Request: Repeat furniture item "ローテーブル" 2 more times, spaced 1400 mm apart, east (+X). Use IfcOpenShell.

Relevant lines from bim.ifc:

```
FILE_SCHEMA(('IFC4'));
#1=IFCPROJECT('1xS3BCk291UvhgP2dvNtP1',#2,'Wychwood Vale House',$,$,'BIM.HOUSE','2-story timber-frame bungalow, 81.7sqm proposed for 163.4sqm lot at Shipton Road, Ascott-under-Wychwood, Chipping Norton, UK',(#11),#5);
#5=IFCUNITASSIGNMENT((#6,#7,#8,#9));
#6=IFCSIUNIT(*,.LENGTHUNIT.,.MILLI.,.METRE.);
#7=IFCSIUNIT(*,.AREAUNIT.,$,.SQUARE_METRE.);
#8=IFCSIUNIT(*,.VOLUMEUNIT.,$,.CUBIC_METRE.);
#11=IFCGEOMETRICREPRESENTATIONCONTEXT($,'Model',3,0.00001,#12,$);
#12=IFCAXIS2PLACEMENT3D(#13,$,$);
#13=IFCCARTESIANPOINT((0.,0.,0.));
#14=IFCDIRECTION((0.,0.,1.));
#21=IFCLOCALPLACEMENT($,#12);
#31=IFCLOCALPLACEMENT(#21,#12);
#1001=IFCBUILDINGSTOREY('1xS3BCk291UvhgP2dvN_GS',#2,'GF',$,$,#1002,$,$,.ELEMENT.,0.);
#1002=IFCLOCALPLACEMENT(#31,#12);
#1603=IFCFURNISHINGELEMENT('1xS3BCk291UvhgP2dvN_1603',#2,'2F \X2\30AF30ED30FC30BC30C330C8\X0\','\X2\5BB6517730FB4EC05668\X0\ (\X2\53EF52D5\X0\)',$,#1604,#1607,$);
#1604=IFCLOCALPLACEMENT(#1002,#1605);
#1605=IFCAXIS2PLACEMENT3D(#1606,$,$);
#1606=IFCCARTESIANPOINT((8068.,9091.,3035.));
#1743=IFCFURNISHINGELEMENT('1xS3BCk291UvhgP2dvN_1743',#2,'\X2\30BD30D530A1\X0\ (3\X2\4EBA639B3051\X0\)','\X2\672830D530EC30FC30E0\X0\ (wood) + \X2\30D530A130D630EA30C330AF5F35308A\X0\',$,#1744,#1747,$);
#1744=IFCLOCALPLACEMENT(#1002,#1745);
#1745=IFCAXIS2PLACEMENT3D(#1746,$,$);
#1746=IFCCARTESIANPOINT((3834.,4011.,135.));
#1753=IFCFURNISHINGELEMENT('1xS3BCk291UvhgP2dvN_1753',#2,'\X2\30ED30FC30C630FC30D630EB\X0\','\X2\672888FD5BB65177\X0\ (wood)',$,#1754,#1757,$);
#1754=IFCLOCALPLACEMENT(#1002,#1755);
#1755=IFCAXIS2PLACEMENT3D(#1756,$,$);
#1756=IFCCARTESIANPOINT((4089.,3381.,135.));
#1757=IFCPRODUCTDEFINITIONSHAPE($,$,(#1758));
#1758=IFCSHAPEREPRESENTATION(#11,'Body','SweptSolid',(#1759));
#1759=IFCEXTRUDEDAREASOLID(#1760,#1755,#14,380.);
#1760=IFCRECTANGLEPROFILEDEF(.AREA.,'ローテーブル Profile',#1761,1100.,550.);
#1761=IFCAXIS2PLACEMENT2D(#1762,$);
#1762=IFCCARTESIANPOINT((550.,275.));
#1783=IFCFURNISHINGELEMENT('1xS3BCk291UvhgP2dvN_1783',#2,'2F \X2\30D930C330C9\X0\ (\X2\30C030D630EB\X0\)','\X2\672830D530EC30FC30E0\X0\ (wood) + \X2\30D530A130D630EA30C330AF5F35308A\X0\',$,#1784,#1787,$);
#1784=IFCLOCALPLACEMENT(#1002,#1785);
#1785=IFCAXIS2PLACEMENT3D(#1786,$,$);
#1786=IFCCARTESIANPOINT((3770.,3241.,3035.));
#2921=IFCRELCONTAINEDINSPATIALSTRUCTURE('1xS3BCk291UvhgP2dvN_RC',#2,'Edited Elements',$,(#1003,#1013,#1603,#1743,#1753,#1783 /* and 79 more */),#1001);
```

```python
import numpy as np
import ifcopenshell
import ifcopenshell.api.geometry
import ifcopenshell.api.root
import ifcopenshell.util.element
import ifcopenshell.util.placement
import ifcopenshell.util.unit

model = ifcopenshell.open("bim.ifc")
unit_scale = ifcopenshell.util.unit.calculate_unit_scale(model)


def reuse_history(source, copy):
    """copy_class also copies each property set's owner history, people and application; keep the originals."""
    for rel in copy.IsDefinedBy:
        if rel.is_a("IfcRelDefinesByProperties") and (history := rel.RelatingPropertyDefinition.OwnerHistory):
            rel.RelatingPropertyDefinition.OwnerHistory = source.OwnerHistory
            ifcopenshell.util.element.remove_deep2(model, history)


source = model.by_id(1753)
base = ifcopenshell.util.placement.get_local_placement(source.ObjectPlacement)
step = np.array([1.0, 0.0, 0.0]) * 1.4 / unit_scale

for i in range(1, 3):
    copy = ifcopenshell.api.root.copy_class(model, product=source)
    copy.Representation = ifcopenshell.util.element.copy_deep(
        model, source.Representation, exclude=["IfcGeometricRepresentationContext", "IfcRepresentationMap"]
    )
    reuse_history(source, copy)
    matrix = base.copy()
    matrix[:3, 3] += i * step
    print("added at", matrix[:3, 3].round(3) + 0.0)
    ifcopenshell.api.geometry.edit_object_placement(model, product=copy, matrix=matrix, is_si=False)

model.write("bim-out.ifc")
```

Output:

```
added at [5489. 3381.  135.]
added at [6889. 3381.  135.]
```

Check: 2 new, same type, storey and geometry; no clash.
